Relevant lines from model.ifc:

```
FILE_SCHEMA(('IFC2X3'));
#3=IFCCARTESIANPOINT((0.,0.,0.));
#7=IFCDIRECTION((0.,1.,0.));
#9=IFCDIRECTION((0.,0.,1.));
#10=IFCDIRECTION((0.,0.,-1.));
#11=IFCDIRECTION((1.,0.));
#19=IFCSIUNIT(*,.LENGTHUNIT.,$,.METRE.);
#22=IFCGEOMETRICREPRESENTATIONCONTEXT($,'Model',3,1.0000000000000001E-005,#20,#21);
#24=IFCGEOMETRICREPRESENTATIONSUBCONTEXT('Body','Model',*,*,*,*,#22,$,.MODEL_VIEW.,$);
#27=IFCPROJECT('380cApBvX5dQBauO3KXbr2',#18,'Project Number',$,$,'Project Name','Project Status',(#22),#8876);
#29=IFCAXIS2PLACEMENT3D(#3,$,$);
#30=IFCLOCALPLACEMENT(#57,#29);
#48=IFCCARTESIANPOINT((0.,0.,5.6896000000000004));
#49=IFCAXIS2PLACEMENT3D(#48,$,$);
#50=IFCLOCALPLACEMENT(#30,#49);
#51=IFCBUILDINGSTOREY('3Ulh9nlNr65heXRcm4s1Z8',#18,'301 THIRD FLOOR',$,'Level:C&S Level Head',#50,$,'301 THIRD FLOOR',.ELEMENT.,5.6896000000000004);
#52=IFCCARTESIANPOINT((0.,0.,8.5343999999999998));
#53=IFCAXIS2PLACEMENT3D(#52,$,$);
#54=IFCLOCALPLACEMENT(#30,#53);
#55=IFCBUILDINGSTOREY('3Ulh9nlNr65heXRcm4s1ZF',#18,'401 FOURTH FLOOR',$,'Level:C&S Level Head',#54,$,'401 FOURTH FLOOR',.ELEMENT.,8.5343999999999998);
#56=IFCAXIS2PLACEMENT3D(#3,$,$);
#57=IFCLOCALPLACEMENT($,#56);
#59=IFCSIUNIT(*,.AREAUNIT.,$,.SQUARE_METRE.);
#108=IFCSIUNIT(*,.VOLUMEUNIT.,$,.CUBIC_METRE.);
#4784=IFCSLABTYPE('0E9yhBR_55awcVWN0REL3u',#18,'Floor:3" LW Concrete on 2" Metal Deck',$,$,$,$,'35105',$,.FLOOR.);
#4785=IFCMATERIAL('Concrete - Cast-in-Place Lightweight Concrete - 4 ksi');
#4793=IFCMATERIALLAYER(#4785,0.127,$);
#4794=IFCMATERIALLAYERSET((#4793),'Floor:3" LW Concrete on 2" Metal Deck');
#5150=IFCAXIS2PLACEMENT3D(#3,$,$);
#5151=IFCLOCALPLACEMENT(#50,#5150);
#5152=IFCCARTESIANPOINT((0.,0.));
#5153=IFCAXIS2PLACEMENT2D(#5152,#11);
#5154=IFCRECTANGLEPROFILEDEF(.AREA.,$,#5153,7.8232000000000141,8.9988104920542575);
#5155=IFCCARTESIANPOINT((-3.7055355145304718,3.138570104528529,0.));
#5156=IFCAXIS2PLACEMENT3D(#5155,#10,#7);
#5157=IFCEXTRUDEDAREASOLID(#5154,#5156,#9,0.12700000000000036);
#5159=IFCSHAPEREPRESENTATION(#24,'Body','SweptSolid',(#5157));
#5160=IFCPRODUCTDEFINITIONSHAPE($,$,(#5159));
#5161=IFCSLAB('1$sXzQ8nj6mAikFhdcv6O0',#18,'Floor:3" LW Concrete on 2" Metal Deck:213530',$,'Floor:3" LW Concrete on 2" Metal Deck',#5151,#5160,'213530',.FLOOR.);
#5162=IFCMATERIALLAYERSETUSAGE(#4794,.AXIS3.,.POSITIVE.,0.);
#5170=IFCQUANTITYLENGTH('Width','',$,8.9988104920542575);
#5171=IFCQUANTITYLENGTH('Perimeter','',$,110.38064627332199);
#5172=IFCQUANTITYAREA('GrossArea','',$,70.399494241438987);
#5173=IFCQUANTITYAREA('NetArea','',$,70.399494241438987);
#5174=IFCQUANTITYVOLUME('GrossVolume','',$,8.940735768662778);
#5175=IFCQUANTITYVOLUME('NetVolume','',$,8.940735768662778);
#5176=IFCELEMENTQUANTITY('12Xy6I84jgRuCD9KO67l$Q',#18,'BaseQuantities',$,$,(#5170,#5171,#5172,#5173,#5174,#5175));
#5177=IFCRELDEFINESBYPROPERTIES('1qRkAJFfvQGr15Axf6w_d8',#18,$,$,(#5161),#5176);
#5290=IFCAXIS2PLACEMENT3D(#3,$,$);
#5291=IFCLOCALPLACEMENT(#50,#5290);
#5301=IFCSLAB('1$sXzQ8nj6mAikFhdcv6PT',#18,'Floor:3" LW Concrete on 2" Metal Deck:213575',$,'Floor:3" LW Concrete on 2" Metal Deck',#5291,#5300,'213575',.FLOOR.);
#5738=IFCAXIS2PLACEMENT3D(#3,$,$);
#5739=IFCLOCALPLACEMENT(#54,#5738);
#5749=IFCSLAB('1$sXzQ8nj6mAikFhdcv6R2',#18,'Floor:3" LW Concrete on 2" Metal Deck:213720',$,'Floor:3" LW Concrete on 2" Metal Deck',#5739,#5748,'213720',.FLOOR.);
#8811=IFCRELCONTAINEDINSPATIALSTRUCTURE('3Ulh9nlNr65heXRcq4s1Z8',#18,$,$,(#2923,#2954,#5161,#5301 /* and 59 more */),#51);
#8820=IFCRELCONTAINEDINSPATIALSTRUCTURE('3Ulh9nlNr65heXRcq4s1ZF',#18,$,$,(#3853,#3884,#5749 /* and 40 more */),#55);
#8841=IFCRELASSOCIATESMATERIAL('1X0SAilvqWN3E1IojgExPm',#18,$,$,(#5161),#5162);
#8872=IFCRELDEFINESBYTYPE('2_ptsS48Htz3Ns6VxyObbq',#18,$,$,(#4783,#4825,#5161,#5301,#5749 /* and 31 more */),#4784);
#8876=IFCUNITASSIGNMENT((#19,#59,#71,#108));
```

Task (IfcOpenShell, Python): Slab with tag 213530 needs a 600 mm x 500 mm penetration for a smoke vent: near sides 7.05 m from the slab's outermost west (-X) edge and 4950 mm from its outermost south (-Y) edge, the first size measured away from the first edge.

```python
import numpy as np
import ifcopenshell
import ifcopenshell.api.feature
import ifcopenshell.api.geometry
import ifcopenshell.api.pset
import ifcopenshell.api.root
import ifcopenshell.geom
import ifcopenshell.util.element
import ifcopenshell.util.placement
import ifcopenshell.util.representation
import ifcopenshell.util.shape
import ifcopenshell.util.unit

model = ifcopenshell.open("model.ifc")
unit_scale = ifcopenshell.util.unit.calculate_unit_scale(model)
area_scale = ifcopenshell.util.unit.calculate_unit_scale(model, "AREAUNIT")
volume_scale = ifcopenshell.util.unit.calculate_unit_scale(model, "VOLUMEUNIT")
settings = ifcopenshell.geom.settings()


def volume(element):
    """Net volume in cubic metres, openings subtracted."""
    shape = ifcopenshell.geom.create_shape(settings, element)
    return ifcopenshell.util.shape.get_volume(shape.geometry)


slab = model.by_id(5161)
before = volume(slab)

# Extent in the slab's own axes, in metres. The edges named are its -X and -Y sides.
slab_shape = ifcopenshell.geom.create_shape(settings, slab)
vertices = ifcopenshell.util.shape.get_vertices(slab_shape.geometry)
x_min, y_min, bottom = vertices.min(axis=0)
top = vertices[:, 2].max()

opening = ifcopenshell.api.root.create_entity(model, ifc_class="IfcOpeningElement", name="Smoke vent opening")
context = ifcopenshell.util.representation.get_context(model, "Model", "Body", "MODEL_VIEW")
width, depth = 0.6, 0.5
outline = [(0.0, 0.0), (width, 0.0), (width, depth), (0.0, depth), (0.0, 0.0)]
# Overshoot both faces by 50 mm so the cut is clean.
shape = ifcopenshell.api.geometry.add_slab_representation(
    model, context=context, depth=top - bottom + 0.1, polyline=outline
)
ifcopenshell.api.geometry.assign_representation(model, product=opening, representation=shape)

matrix = ifcopenshell.util.placement.get_local_placement(slab.ObjectPlacement)
matrix[:, 3] = matrix @ np.append(np.array([x_min + 7.05, y_min + 4.95, bottom - 0.05]) / unit_scale, 1.0)
ifcopenshell.api.geometry.edit_object_placement(model, product=opening, matrix=matrix, is_si=False)
ifcopenshell.api.feature.add_feature(model, feature=opening, element=slab)

after = volume(slab)

# Update the slab's stored quantities.
qto = model.by_id(ifcopenshell.util.element.get_pset(slab, "BaseQuantities", should_inherit=False)["id"])
ifcopenshell.api.pset.edit_qto(model, qto=qto, properties={
    "NetArea": after / (top - bottom) / area_scale,
    "NetVolume": after / volume_scale,
})

print(f"slab volume {before:.3f} -> {after:.3f} m3")

model.write("model-out.ifc")
```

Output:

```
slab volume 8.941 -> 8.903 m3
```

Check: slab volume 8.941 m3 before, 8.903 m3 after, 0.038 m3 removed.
